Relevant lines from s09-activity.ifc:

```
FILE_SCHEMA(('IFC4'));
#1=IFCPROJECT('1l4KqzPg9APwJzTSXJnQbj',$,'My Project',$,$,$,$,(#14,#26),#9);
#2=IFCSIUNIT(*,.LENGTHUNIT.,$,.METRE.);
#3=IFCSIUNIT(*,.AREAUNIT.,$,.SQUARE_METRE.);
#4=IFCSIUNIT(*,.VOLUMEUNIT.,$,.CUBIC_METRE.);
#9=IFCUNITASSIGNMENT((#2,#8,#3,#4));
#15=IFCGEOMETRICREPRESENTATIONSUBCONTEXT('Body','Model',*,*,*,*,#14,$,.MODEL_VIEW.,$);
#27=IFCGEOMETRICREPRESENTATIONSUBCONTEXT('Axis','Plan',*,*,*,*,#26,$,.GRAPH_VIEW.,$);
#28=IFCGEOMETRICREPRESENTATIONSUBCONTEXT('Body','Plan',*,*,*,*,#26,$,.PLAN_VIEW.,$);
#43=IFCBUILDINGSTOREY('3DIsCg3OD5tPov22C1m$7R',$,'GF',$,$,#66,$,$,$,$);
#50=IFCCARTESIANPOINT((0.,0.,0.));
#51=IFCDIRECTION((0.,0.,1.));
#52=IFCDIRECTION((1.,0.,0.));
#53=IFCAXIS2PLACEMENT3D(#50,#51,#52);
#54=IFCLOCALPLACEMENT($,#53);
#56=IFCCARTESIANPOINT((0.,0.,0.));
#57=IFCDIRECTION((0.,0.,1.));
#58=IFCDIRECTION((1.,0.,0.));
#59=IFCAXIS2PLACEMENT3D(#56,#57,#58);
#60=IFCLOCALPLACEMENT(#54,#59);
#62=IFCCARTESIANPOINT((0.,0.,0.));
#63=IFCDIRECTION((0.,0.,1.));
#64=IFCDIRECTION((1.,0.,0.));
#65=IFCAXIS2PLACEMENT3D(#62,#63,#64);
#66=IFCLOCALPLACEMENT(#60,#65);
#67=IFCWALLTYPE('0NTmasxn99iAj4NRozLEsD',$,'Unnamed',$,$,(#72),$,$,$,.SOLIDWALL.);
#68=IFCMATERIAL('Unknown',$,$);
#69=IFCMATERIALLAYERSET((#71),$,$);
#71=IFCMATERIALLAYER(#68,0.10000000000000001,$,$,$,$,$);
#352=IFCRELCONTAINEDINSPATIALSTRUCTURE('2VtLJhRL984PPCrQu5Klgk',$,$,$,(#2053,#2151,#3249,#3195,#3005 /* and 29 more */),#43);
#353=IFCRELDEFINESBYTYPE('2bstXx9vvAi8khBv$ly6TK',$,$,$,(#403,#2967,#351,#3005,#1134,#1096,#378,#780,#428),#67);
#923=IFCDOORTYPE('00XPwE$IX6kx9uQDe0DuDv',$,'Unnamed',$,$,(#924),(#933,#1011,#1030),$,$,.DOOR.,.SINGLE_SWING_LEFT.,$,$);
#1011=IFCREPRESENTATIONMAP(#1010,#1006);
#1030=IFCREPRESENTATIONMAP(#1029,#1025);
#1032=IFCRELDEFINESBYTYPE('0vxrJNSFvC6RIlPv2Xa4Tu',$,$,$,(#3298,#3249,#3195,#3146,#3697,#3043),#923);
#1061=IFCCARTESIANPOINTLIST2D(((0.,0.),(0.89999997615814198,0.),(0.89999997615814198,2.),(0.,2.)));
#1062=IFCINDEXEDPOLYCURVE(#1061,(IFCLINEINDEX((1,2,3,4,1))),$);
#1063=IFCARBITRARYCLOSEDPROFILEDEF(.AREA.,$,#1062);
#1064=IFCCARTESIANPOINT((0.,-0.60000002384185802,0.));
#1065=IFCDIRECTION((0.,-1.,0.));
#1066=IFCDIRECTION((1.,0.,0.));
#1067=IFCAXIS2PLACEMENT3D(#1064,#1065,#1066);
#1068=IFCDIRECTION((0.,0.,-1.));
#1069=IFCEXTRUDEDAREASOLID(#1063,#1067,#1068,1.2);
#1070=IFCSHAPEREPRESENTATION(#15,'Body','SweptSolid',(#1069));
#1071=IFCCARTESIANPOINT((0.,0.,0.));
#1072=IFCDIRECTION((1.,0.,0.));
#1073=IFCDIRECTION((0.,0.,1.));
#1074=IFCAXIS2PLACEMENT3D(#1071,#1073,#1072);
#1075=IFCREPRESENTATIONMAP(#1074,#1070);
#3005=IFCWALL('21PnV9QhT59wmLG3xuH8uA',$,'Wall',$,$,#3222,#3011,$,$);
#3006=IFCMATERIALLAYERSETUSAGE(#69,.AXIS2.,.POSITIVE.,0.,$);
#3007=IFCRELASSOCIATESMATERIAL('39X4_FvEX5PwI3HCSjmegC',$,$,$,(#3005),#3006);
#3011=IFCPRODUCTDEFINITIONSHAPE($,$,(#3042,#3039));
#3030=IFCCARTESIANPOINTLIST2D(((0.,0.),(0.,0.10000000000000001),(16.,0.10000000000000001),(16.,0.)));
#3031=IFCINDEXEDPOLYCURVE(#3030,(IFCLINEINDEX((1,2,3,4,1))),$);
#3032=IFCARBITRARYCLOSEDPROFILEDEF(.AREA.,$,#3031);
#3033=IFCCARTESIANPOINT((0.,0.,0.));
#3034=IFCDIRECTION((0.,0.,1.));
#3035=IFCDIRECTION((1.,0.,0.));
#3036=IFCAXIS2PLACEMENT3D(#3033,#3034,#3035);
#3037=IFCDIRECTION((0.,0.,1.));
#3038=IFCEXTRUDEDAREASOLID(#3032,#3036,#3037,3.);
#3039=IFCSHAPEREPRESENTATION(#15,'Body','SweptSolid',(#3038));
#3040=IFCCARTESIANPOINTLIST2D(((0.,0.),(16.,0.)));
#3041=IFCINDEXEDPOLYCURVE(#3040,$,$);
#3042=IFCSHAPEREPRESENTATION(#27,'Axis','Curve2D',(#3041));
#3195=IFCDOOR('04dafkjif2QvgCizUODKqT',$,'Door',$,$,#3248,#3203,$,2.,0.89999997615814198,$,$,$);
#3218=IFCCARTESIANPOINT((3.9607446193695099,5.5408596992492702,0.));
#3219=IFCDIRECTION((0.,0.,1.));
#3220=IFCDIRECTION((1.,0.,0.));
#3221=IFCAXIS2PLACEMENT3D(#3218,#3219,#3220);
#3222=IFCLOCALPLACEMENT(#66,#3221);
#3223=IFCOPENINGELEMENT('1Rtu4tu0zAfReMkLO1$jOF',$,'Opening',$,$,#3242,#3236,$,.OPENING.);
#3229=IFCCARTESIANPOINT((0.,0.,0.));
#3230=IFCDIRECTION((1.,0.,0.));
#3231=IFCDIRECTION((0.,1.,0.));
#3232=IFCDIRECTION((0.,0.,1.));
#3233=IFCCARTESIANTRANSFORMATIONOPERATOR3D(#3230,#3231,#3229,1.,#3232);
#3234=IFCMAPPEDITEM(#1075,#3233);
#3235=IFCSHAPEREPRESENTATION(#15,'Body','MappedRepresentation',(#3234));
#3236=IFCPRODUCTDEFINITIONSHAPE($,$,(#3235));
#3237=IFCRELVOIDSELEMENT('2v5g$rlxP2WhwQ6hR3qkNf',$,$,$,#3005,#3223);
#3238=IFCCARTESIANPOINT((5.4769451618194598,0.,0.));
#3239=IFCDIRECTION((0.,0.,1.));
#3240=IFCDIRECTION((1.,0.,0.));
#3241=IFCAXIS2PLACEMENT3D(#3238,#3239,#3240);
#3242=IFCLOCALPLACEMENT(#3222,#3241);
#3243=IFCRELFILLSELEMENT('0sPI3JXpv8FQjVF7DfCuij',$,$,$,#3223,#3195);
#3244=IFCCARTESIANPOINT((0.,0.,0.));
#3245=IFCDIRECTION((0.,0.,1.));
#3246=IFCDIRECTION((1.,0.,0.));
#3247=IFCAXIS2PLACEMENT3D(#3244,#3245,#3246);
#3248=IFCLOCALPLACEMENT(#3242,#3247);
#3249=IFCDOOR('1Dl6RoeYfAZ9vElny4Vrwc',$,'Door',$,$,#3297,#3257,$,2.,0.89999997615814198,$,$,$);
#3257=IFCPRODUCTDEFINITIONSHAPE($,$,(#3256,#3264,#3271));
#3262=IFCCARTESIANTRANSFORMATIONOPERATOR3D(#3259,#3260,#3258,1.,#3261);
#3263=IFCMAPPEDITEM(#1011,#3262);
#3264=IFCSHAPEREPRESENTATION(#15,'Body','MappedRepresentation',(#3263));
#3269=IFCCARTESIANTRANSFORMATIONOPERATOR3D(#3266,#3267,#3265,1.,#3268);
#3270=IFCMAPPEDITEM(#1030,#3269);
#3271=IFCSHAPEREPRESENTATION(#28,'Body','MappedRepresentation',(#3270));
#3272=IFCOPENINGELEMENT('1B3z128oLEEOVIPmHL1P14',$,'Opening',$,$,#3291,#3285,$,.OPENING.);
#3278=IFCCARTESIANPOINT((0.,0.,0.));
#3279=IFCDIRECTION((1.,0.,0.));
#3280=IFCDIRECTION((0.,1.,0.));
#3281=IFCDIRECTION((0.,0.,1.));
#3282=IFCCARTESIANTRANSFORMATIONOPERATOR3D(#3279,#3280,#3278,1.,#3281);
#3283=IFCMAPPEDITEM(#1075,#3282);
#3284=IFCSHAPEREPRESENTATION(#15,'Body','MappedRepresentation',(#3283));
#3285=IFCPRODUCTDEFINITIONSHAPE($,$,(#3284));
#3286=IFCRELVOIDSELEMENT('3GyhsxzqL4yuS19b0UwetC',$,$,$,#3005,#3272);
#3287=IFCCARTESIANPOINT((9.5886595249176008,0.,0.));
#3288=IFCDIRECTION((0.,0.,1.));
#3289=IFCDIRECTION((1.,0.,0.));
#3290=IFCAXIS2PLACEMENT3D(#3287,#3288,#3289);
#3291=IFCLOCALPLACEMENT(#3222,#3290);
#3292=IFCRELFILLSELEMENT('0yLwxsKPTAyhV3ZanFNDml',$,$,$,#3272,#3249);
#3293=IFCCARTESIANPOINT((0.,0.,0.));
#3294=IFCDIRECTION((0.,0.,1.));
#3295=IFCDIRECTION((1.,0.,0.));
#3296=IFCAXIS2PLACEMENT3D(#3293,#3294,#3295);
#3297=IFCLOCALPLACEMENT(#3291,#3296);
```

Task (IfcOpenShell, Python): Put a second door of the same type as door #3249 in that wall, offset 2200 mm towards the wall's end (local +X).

```python
import ifcopenshell
import ifcopenshell.api.feature
import ifcopenshell.api.geometry
import ifcopenshell.api.root
import ifcopenshell.geom
import ifcopenshell.util.element
import ifcopenshell.util.placement
import ifcopenshell.util.shape
import ifcopenshell.util.unit

model = ifcopenshell.open("s09-activity.ifc")
unit_scale = ifcopenshell.util.unit.calculate_unit_scale(model)
settings = ifcopenshell.geom.settings()


def volume(element):
    """Net volume in cubic metres, openings subtracted."""
    shape = ifcopenshell.geom.create_shape(settings, element)
    return ifcopenshell.util.shape.get_volume(shape.geometry)


door = model.by_guid("1Dl6RoeYfAZ9vElny4Vrwc")
opening = door.FillsVoids[0].RelatingOpeningElement
wall = opening.VoidsElements[0].RelatingBuildingElement
before = volume(wall)
shift = ifcopenshell.util.placement.get_local_placement(wall.ObjectPlacement)[:3, 0] * 2.2 / unit_scale

# copy_class copies the void relationship, type, container and properties, but no geometry.
new_opening = ifcopenshell.api.root.copy_class(model, product=opening)
new_opening.Representation = ifcopenshell.util.element.copy_deep(
    model, opening.Representation, exclude=["IfcGeometricRepresentationContext", "IfcRepresentationMap"]
)
new_door = ifcopenshell.api.root.copy_class(model, product=door)
new_door.Representation = ifcopenshell.util.element.copy_deep(
    model, door.Representation, exclude=["IfcGeometricRepresentationContext", "IfcRepresentationMap"]
)
ifcopenshell.api.feature.add_filling(model, opening=new_opening, element=new_door)

for old, new in ((opening, new_opening), (door, new_door)):
    matrix = ifcopenshell.util.placement.get_local_placement(old.ObjectPlacement)
    matrix[:3, 3] += shift
    ifcopenshell.api.geometry.edit_object_placement(model, product=new, matrix=matrix, is_si=False)

after = volume(wall)

print(f"wall volume {before:.3f} -> {after:.3f} m3")

model.write("s09-activity_updated.ifc")
```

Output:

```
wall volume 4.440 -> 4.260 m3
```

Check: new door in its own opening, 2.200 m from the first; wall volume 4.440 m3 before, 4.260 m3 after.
